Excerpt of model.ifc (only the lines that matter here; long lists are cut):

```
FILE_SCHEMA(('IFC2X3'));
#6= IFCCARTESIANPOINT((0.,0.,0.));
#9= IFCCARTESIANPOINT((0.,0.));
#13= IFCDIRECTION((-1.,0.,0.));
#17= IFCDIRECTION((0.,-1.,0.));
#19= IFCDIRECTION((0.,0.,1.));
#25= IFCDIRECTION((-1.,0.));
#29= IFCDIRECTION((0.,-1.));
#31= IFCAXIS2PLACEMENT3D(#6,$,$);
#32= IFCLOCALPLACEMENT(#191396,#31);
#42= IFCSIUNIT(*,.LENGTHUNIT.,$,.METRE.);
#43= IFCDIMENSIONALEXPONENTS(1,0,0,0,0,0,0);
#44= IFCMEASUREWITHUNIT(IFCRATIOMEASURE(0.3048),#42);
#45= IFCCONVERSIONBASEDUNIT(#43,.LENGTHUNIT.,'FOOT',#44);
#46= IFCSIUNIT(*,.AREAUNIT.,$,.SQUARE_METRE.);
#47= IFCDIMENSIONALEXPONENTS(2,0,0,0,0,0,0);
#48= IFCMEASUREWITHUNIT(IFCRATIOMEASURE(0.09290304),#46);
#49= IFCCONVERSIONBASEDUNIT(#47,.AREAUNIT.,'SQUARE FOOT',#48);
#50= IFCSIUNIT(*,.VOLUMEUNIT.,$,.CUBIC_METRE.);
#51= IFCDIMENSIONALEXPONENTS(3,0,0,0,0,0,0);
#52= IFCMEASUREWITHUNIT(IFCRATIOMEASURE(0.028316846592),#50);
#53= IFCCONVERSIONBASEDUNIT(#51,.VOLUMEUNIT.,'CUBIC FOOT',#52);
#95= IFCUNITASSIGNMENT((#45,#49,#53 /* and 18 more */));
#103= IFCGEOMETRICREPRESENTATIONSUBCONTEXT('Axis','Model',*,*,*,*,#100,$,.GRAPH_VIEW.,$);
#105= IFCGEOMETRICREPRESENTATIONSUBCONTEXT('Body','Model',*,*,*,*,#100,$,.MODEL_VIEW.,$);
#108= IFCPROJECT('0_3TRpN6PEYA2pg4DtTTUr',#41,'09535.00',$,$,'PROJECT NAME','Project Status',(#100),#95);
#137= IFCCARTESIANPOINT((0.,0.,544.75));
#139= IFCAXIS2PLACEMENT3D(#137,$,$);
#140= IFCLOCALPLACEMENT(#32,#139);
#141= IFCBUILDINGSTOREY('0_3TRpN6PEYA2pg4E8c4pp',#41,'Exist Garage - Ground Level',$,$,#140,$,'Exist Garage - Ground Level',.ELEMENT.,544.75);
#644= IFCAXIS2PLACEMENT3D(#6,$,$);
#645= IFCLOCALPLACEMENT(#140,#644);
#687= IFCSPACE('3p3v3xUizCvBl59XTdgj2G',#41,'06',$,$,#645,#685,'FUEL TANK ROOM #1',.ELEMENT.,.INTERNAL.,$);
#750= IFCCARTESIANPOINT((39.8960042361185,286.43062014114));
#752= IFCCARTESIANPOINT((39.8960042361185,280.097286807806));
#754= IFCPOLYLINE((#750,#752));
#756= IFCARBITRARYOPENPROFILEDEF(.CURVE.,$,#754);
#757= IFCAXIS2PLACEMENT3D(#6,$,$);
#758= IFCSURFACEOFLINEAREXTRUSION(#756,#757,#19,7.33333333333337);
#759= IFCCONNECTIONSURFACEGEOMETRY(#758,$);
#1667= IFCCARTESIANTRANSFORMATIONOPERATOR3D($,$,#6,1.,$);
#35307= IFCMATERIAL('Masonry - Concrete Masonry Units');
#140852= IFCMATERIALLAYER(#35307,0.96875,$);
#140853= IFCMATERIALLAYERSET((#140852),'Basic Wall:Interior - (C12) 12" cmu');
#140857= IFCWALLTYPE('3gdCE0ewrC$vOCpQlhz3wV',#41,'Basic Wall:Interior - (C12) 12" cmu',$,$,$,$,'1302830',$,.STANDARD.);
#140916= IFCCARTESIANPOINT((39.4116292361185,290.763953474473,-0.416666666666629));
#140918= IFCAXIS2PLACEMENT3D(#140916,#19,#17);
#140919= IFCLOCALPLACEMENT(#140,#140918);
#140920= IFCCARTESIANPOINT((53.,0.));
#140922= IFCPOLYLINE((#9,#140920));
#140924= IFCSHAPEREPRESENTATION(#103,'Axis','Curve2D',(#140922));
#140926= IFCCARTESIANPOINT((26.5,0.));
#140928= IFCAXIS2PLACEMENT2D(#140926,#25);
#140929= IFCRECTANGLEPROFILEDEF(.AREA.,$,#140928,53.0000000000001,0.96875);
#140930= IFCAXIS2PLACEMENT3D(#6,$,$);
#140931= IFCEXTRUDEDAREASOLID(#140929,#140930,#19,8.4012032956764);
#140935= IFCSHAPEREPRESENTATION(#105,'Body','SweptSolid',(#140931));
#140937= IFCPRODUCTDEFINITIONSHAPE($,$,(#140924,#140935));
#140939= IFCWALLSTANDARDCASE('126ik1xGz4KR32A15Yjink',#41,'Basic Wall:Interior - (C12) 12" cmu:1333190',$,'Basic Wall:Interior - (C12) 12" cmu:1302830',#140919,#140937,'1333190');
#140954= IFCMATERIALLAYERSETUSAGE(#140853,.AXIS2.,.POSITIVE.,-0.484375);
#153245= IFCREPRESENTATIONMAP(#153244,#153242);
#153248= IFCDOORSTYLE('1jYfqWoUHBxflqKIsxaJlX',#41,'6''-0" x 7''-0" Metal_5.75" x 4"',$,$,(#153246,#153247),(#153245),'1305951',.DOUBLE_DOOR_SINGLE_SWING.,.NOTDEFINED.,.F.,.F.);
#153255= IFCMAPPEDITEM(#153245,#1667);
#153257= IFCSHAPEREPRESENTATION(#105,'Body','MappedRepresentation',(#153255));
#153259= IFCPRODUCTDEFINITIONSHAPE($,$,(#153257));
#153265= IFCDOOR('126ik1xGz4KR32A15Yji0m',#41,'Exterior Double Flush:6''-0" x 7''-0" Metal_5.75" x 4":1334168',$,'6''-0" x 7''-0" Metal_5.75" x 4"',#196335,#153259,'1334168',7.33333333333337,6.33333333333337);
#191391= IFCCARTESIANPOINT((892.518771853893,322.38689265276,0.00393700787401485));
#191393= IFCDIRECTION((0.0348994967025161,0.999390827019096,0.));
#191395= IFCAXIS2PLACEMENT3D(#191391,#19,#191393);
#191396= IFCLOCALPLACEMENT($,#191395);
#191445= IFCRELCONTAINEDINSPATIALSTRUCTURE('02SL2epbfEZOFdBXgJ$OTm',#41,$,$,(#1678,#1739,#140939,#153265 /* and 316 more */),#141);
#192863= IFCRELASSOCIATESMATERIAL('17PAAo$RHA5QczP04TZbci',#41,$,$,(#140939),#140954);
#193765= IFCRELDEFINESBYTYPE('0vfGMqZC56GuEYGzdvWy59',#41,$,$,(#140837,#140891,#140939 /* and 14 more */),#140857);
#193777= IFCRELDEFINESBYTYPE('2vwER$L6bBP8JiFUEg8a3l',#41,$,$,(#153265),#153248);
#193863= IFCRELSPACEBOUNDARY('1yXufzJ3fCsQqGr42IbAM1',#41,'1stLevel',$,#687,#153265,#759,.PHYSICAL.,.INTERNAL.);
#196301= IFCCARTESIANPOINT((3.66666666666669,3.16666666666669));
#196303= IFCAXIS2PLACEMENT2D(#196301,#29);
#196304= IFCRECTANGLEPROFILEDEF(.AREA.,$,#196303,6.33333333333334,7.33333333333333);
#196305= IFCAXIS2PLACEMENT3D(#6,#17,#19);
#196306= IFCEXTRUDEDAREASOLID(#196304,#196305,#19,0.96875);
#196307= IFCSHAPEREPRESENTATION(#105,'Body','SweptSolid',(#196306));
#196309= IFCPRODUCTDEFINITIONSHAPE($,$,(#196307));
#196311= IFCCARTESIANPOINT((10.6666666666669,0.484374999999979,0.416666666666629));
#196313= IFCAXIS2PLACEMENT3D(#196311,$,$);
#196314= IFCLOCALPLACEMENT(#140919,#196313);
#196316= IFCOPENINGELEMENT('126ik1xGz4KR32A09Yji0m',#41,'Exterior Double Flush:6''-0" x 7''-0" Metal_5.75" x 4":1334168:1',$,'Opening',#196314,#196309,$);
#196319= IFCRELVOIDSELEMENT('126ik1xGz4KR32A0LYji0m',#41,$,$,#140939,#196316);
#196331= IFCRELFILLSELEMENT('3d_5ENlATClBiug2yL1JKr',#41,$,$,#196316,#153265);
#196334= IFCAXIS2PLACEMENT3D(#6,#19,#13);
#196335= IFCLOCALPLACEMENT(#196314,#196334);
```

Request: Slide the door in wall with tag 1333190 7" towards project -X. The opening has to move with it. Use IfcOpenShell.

```python
import numpy as np
import ifcopenshell
import ifcopenshell.api.geometry
import ifcopenshell.util.placement
import ifcopenshell.util.unit

model = ifcopenshell.open("model.ifc")
unit_scale = ifcopenshell.util.unit.calculate_unit_scale(model)

door = model.by_guid("126ik1xGz4KR32A15Yji0m")
opening = door.FillsVoids[0].RelatingOpeningElement
wall = opening.VoidsElements[0].RelatingBuildingElement

wall_matrix = ifcopenshell.util.placement.get_local_placement(wall.ObjectPlacement)
shift = wall_matrix[:3, 0] * -7 * 0.0254 / unit_scale
before = ifcopenshell.util.placement.get_local_placement(door.ObjectPlacement)[:3, 3].copy()

# The door is placed relative to its opening, so it follows when the opening moves.
matrix = ifcopenshell.util.placement.get_local_placement(opening.ObjectPlacement)
matrix[:3, 3] += shift
ifcopenshell.api.geometry.edit_object_placement(
    model, product=opening, matrix=matrix, is_si=False, should_transform_children=True
)

# Space boundary surfaces are stored in each space's coordinates; move them too.
for rel in door.ProvidesBoundaries:
    if not rel.ConnectionGeometry:
        continue
    surface = rel.ConnectionGeometry.SurfaceOnRelatingElement
    space_matrix = ifcopenshell.util.placement.get_local_placement(rel.RelatingSpace.ObjectPlacement)
    point = np.array(surface.Position.Location.Coordinates) + space_matrix[:3, :3].T @ shift
    surface.Position = model.createIfcAxis2Placement3D(
        model.createIfcCartesianPoint(point.tolist()), surface.Position.Axis, surface.Position.RefDirection
    )

after = ifcopenshell.util.placement.get_local_placement(door.ObjectPlacement)[:3, 3]
print("door moved by", (after - before).round(3) + 0.0)

model.write("model-out.ifc")
```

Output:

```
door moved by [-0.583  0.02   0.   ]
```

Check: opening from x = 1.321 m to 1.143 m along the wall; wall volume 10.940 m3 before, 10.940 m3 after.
